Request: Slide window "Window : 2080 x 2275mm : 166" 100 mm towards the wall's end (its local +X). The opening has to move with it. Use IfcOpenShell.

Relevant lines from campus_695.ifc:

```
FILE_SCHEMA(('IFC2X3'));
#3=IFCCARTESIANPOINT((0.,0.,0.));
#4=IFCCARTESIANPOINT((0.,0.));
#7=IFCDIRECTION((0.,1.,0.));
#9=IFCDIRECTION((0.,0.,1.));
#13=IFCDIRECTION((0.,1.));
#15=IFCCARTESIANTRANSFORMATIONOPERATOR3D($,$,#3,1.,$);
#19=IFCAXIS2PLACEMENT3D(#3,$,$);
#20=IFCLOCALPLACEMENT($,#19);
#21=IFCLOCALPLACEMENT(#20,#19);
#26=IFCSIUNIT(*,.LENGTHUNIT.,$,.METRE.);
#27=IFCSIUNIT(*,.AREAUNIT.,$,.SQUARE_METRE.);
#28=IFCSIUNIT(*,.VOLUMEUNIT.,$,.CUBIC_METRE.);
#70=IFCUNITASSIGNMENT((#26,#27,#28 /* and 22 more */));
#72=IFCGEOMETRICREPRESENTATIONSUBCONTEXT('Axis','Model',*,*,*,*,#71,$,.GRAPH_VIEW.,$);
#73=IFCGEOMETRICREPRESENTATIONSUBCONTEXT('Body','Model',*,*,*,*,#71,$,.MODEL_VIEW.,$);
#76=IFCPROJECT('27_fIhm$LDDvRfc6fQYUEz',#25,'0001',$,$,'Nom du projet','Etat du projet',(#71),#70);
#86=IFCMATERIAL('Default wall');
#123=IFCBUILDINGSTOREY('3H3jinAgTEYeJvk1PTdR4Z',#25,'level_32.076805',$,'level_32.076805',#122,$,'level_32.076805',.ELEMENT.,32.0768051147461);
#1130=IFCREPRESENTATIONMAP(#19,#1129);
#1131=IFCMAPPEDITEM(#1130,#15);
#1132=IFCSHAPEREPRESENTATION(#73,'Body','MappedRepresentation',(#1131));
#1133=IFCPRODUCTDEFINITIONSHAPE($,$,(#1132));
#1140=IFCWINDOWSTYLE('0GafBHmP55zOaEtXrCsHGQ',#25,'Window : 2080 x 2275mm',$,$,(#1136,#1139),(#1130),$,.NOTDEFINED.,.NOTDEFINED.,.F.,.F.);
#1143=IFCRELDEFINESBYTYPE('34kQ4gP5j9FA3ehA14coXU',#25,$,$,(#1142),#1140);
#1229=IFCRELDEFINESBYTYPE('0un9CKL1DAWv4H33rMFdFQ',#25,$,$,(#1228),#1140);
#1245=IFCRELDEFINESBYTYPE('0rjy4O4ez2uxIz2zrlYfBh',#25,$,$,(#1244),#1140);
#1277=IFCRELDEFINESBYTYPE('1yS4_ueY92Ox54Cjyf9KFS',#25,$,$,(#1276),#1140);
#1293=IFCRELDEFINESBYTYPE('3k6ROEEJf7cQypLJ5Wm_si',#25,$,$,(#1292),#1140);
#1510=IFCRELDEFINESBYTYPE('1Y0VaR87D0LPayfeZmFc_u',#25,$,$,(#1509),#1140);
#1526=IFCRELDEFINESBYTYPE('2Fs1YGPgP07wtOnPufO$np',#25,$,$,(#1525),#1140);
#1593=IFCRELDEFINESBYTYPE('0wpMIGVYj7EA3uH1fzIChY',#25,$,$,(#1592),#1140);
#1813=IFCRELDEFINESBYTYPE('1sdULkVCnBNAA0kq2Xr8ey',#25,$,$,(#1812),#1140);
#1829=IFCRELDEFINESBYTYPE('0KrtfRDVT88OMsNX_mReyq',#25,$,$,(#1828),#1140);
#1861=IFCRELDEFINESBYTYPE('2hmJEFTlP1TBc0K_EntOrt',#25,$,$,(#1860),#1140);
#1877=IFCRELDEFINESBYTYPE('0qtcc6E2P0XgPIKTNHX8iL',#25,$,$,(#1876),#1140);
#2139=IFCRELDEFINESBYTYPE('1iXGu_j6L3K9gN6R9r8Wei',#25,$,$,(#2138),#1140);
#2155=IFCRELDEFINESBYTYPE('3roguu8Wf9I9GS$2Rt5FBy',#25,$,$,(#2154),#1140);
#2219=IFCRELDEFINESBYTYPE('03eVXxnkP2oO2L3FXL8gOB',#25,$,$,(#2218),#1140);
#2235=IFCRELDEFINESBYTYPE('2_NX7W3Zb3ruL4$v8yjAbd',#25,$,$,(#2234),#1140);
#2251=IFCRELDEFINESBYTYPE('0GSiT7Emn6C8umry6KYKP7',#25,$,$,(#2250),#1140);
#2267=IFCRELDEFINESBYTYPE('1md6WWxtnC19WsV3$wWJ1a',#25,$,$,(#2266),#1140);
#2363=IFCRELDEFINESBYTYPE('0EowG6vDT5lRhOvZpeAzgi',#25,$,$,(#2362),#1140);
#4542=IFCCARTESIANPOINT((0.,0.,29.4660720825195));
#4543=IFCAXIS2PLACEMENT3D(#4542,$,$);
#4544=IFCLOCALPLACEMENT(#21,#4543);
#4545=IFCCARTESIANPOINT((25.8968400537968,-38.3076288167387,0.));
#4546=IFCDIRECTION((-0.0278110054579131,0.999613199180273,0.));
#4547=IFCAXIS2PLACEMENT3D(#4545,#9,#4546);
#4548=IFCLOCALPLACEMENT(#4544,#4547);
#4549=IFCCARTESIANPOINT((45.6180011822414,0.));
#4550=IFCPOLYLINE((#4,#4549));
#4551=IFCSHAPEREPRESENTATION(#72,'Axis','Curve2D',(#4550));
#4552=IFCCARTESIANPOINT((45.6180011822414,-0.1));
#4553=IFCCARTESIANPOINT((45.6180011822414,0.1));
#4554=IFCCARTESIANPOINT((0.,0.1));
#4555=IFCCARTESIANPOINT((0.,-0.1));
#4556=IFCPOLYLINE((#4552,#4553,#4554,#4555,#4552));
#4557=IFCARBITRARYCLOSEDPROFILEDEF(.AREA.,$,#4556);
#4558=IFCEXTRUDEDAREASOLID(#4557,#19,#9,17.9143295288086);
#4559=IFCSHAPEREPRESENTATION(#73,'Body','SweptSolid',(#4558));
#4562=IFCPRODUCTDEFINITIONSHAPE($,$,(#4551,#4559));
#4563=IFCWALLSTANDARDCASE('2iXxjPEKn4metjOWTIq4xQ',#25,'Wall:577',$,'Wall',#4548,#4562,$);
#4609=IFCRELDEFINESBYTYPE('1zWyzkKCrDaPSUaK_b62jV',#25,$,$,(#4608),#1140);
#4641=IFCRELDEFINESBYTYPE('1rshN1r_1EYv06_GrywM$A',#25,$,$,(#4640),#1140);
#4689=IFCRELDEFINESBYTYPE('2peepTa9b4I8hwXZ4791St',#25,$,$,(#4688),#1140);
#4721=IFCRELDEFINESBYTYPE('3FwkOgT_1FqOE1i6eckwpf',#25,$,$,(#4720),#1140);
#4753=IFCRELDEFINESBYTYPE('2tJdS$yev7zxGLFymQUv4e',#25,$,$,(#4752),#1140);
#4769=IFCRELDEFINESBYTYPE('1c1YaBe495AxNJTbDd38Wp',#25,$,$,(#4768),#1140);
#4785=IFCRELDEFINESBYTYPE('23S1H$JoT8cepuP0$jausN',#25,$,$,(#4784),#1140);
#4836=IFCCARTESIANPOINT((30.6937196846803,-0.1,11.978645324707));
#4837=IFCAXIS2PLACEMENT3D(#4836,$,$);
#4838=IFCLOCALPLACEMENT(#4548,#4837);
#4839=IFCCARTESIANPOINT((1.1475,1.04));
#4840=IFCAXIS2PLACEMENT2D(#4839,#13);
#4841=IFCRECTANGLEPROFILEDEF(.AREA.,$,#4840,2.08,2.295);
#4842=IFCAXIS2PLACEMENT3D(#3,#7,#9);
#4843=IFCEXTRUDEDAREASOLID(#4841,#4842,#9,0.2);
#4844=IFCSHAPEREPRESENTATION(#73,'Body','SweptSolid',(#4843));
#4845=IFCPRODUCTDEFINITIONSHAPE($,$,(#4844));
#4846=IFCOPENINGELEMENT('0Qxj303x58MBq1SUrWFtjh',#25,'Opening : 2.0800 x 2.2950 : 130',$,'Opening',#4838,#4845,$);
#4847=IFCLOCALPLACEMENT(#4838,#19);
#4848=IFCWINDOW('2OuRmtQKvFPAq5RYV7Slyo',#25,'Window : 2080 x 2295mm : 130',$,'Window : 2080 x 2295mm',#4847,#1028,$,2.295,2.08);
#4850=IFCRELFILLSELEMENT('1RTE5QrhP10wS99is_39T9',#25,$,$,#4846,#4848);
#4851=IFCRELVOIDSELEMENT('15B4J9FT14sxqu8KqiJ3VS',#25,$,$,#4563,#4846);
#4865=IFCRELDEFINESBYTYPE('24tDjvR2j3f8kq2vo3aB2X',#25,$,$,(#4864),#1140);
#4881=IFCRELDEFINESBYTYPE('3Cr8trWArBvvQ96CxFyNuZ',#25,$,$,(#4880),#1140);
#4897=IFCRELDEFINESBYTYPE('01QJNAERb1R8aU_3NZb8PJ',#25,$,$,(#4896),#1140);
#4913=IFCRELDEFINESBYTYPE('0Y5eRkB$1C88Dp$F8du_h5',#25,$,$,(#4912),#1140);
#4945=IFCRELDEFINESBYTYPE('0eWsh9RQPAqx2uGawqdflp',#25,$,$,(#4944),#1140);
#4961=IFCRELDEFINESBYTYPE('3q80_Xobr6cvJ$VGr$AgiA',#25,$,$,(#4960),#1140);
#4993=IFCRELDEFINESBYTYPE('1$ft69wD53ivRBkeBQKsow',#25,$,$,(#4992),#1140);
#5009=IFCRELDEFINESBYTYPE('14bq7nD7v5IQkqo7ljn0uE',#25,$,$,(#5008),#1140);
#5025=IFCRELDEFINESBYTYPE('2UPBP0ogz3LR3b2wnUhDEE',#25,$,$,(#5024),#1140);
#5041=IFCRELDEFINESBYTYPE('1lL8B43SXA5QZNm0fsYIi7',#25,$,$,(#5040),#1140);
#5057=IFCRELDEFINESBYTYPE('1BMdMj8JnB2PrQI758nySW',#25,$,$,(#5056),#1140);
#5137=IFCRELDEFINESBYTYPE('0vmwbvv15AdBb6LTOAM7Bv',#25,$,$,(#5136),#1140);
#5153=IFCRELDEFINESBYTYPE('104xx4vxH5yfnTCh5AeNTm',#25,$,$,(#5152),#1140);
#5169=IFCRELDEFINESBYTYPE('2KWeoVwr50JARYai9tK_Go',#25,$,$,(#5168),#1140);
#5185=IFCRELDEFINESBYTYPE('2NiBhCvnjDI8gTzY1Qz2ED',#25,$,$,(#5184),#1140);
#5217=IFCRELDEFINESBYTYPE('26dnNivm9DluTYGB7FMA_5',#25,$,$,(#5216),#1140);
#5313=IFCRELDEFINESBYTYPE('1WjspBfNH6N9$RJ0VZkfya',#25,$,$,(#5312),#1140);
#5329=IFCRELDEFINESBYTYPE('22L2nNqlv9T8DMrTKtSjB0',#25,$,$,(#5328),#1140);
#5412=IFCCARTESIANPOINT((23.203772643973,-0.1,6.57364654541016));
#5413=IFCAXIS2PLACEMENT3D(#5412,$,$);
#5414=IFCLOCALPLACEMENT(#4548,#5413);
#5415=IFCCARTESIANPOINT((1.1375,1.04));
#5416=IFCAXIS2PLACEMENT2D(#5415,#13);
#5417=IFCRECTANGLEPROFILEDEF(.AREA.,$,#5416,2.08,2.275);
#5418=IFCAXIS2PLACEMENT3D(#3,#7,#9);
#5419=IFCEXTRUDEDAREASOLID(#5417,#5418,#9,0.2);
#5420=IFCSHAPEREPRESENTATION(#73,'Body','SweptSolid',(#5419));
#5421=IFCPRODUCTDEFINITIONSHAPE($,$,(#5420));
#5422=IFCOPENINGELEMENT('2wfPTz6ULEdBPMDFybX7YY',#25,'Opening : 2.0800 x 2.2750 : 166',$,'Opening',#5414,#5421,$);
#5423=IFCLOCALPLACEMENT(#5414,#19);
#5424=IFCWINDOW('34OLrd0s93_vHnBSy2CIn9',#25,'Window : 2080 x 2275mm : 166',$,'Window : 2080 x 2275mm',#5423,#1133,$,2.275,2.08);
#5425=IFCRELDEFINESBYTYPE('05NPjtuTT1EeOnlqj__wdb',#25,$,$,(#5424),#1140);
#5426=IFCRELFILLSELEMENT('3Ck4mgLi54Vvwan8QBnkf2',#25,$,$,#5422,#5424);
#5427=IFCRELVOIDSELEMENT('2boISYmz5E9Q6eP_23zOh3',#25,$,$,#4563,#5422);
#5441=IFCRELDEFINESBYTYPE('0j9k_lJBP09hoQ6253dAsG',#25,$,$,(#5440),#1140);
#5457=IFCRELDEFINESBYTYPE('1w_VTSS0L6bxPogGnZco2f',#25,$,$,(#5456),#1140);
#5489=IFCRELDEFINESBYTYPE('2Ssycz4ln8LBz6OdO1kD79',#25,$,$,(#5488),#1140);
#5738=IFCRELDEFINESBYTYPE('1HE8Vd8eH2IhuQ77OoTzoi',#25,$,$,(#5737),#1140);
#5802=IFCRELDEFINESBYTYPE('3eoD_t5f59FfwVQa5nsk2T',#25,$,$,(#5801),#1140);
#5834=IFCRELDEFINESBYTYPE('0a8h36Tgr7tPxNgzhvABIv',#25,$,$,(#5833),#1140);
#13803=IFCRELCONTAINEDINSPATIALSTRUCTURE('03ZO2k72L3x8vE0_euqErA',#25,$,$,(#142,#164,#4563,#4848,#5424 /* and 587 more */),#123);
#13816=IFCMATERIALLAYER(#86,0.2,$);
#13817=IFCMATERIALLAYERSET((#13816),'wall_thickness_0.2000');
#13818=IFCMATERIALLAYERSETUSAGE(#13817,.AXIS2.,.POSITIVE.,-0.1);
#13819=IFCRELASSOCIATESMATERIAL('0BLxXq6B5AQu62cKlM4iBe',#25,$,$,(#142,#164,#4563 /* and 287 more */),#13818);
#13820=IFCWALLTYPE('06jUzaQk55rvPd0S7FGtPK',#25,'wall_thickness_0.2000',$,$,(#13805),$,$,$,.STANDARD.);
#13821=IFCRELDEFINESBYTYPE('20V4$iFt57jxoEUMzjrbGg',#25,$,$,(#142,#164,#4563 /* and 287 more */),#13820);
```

```python
import ifcopenshell
import ifcopenshell.api.geometry
import ifcopenshell.util.placement
import ifcopenshell.util.unit

model = ifcopenshell.open("campus_695.ifc")
unit_scale = ifcopenshell.util.unit.calculate_unit_scale(model)

window = model.by_guid("34OLrd0s93_vHnBSy2CIn9")
opening = window.FillsVoids[0].RelatingOpeningElement
wall = opening.VoidsElements[0].RelatingBuildingElement

wall_matrix = ifcopenshell.util.placement.get_local_placement(wall.ObjectPlacement)
shift = wall_matrix[:3, 0] * 0.1 / unit_scale
before = ifcopenshell.util.placement.get_local_placement(window.ObjectPlacement)[:3, 3].copy()

# The window is placed relative to its opening, so it follows when the opening moves.
matrix = ifcopenshell.util.placement.get_local_placement(opening.ObjectPlacement)
matrix[:3, 3] += shift
ifcopenshell.api.geometry.edit_object_placement(
    model, product=opening, matrix=matrix, is_si=False, should_transform_children=True
)

after = ifcopenshell.util.placement.get_local_placement(window.ObjectPlacement)[:3, 3]
print("window moved by", (after - before).round(3) + 0.0)

model.write("campus_695_rev.ifc")
```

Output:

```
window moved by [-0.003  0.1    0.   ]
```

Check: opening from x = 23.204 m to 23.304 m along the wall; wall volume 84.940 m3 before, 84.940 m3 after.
